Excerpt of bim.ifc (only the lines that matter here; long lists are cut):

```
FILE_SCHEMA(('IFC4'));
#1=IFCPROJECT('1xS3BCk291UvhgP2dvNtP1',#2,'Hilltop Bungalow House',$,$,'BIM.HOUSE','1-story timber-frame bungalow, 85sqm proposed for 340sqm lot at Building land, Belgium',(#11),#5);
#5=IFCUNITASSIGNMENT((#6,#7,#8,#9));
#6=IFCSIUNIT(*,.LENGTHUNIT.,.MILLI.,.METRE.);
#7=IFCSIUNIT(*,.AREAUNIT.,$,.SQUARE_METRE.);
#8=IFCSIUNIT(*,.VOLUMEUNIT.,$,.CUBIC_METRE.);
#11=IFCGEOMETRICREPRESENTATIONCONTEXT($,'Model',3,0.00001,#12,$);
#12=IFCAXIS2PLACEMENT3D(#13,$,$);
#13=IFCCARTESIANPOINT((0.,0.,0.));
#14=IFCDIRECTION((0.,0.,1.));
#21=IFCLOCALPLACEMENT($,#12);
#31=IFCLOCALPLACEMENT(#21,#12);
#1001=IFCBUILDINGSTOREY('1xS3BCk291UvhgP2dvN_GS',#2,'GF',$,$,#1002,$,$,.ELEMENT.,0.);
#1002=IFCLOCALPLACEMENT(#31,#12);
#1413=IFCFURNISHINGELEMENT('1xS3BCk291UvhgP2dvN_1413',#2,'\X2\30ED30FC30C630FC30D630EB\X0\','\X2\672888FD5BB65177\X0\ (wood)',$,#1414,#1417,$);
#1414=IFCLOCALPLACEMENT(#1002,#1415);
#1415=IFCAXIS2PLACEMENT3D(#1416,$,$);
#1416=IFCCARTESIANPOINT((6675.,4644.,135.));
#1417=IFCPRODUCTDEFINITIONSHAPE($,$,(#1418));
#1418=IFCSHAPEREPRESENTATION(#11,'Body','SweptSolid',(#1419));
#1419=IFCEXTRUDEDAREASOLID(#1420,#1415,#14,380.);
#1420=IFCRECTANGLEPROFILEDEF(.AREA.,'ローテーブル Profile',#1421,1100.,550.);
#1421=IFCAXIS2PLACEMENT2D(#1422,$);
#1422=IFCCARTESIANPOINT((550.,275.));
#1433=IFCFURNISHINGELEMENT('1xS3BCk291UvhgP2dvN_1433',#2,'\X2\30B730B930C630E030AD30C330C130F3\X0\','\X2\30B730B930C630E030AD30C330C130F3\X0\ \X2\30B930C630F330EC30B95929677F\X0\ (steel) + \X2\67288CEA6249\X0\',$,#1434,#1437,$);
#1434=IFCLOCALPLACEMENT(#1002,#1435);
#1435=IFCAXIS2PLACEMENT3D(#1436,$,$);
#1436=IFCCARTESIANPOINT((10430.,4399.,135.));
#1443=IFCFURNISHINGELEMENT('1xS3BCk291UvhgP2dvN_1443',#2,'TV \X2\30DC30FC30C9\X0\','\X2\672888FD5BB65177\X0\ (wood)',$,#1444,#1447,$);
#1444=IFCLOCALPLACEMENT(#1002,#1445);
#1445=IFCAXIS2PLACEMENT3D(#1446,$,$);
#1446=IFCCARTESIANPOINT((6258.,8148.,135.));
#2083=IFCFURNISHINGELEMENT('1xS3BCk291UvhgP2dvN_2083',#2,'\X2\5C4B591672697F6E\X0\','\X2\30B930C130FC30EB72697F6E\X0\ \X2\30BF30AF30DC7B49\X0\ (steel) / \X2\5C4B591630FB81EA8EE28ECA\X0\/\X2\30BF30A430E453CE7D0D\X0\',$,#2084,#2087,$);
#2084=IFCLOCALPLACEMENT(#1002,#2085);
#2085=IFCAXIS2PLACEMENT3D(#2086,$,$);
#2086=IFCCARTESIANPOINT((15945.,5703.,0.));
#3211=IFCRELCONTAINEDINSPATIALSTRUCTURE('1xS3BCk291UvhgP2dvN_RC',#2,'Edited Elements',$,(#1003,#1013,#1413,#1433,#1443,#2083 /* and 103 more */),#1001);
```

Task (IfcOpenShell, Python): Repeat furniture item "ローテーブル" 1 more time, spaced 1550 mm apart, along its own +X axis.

```python
import ifcopenshell
import ifcopenshell.api.geometry
import ifcopenshell.api.root
import ifcopenshell.util.element
import ifcopenshell.util.placement
import ifcopenshell.util.unit

model = ifcopenshell.open("bim.ifc")
unit_scale = ifcopenshell.util.unit.calculate_unit_scale(model)


def reuse_history(source, copy):
    """copy_class also copies each property set's owner history, people and application; keep the originals."""
    for rel in copy.IsDefinedBy:
        if rel.is_a("IfcRelDefinesByProperties") and (history := rel.RelatingPropertyDefinition.OwnerHistory):
            rel.RelatingPropertyDefinition.OwnerHistory = source.OwnerHistory
            ifcopenshell.util.element.remove_deep2(model, history)


source = model.by_guid("1xS3BCk291UvhgP2dvN_1413")
base = ifcopenshell.util.placement.get_local_placement(source.ObjectPlacement)
step = base[:3, 0] * 1.55 / unit_scale

for i in range(1, 2):
    copy = ifcopenshell.api.root.copy_class(model, product=source)
    copy.Representation = ifcopenshell.util.element.copy_deep(
        model, source.Representation, exclude=["IfcGeometricRepresentationContext", "IfcRepresentationMap"]
    )
    reuse_history(source, copy)
    matrix = base.copy()
    matrix[:3, 3] += i * step
    print("added at", matrix[:3, 3].round(3) + 0.0)
    ifcopenshell.api.geometry.edit_object_placement(model, product=copy, matrix=matrix, is_si=False)

model.write("bim_rev.ifc")
```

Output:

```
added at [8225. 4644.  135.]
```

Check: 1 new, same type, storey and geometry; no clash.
